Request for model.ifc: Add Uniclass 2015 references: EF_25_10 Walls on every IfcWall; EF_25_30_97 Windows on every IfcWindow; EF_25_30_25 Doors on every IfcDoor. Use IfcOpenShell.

First a look at what the model holds.

```python
import ifcopenshell

model = ifcopenshell.open("model.ifc")
print(model.schema)
print("classifications:", [c.Name for c in model.by_type("IfcClassification")])
for ifc_class in ("IfcDoor", "IfcRoof", "IfcStair", "IfcWall", "IfcWindow"):
    print(ifc_class, len(model.by_type(ifc_class)))
```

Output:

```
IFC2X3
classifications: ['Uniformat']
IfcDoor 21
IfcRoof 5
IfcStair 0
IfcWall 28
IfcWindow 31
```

```python
import ifcopenshell
import ifcopenshell.api.classification

model = ifcopenshell.open("model.ifc")

# IFC2X3 requires Source and Edition and has no link from the project to the system.
system = model.create_entity("IfcClassification", Source="NBS", Edition="2015", Name="Uniclass 2015")

codes = {
    "IfcWall": ("EF_25_10", "Walls"),
    "IfcWindow": ("EF_25_30_97", "Windows"),
    "IfcDoor": ("EF_25_30_25", "Doors"),
}
for ifc_class, (code, name) in codes.items():
    products = model.by_type(ifc_class)
    ifcopenshell.api.classification.add_reference(
        model, products=products, classification=system, identification=code, name=name
    )
    print(code, len(products))

model.write("model_updated.ifc")
```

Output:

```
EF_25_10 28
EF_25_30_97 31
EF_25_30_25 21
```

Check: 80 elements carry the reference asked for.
